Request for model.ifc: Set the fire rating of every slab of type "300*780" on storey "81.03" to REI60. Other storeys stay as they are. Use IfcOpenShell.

First a look at what the model holds.

```python
import ifcopenshell
import ifcopenshell.util.element

model = ifcopenshell.open("model.ifc")
print(model.schema)
storey = next(s for s in model.by_type("IfcBuildingStorey") if s.Name == "81.03")
slabs = [e for e in ifcopenshell.util.element.get_decomposition(storey) if e.is_a("IfcSlab")]
seen = {}
for e in slabs:
    element_type = ifcopenshell.util.element.get_type(e)
    key = (element_type.Name if element_type != e and element_type else None, ifcopenshell.util.element.get_pset(e, "Pset_SlabCommon", "FireRating"))
    seen[key] = seen.get(key, 0) + 1
for (name, value), count in sorted(seen.items(), key=str):
    print(count, "x", name, "|", value)
```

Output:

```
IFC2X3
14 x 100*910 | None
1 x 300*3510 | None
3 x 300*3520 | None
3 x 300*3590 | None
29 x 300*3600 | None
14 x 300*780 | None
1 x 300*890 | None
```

```python
import ifcopenshell
import ifcopenshell.api.pset
import ifcopenshell.util.element

model = ifcopenshell.open("model.ifc")

storey = next(s for s in model.by_type("IfcBuildingStorey") if s.Name == "81.03")
slabs = [e for e in ifcopenshell.util.element.get_decomposition(storey) if e.is_a("IfcSlab")]

count = 0
for e in slabs:
    element_type = ifcopenshell.util.element.get_type(e)
    if element_type in (None, e) or element_type.Name != "300*780":
        continue
    found = ifcopenshell.util.element.get_pset(e, "Pset_SlabCommon", should_inherit=False)
    if found:
        pset = model.by_id(found["id"])
        if len(ifcopenshell.util.element.get_elements_by_pset(pset)) > 1:
            pset = ifcopenshell.api.pset.unshare_pset(model, products=[e], pset=pset)[0]
    else:
        pset = ifcopenshell.api.pset.add_pset(model, product=e, name="Pset_SlabCommon")
    ifcopenshell.api.pset.edit_pset(model, pset=pset, properties={"FireRating": "REI60"})
    count += 1

print(count, "slabs updated")

model.write("model-out.ifc")
```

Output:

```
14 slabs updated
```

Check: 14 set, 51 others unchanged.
